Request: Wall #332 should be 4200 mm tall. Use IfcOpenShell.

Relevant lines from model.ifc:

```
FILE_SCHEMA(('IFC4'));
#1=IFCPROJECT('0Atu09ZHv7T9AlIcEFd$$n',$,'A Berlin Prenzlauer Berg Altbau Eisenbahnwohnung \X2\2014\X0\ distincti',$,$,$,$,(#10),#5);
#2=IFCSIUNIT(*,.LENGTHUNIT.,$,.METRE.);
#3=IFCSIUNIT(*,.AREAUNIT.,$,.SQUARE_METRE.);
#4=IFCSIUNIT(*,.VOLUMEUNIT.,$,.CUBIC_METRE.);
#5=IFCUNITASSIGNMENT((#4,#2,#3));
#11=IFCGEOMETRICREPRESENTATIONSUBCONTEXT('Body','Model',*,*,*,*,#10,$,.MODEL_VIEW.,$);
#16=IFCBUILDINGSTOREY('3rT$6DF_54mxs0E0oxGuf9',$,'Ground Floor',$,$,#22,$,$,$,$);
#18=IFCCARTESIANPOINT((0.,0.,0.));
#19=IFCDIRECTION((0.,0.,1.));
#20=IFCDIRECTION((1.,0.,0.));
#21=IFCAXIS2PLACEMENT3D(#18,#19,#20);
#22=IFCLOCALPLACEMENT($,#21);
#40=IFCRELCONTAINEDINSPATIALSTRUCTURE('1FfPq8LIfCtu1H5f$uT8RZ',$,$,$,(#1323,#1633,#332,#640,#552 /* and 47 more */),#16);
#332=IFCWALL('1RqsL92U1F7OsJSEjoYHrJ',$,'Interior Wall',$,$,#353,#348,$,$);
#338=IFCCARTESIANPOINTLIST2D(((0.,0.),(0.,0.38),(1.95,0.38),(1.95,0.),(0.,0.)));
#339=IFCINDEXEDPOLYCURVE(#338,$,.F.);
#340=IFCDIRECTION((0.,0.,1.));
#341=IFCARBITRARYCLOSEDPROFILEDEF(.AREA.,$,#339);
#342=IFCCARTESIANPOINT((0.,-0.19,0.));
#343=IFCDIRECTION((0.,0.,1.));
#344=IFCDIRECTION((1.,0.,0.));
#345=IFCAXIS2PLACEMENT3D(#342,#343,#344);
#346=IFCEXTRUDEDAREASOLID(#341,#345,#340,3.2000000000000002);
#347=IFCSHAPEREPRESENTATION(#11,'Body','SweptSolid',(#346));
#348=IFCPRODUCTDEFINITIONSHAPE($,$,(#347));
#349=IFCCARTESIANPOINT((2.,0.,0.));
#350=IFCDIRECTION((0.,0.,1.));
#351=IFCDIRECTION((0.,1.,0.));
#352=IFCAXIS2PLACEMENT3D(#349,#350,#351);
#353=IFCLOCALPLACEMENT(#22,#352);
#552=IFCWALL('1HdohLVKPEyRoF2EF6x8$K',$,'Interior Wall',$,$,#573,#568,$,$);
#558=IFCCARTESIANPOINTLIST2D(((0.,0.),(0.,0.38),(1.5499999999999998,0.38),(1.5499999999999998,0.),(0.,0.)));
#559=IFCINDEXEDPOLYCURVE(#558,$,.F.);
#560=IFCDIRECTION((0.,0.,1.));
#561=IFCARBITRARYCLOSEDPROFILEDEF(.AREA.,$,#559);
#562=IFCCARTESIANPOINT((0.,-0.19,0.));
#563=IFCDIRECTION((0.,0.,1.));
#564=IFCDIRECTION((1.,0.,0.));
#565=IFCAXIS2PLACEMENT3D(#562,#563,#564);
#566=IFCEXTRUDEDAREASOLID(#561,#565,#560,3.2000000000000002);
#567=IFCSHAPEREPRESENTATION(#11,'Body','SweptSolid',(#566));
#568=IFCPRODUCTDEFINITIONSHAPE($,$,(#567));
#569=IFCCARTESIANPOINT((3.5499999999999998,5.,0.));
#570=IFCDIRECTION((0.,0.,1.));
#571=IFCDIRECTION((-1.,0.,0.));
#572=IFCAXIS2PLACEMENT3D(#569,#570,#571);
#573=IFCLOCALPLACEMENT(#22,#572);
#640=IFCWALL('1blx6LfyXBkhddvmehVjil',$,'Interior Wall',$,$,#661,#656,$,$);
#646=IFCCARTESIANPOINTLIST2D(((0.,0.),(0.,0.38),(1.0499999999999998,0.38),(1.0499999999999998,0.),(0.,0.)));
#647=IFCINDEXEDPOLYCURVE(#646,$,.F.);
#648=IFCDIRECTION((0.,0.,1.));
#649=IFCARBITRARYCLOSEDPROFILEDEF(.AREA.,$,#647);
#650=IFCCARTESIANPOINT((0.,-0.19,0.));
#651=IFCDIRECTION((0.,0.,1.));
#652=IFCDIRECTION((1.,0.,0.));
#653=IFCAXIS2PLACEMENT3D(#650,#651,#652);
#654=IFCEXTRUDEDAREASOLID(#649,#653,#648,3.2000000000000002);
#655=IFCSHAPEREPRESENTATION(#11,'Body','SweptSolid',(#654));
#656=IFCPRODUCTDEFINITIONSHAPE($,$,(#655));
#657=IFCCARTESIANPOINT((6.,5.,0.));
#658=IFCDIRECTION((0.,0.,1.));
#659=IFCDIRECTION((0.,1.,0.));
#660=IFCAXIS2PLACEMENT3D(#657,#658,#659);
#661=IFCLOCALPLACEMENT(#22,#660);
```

```python
import ifcopenshell
import ifcopenshell.geom
import ifcopenshell.util.representation
import ifcopenshell.util.shape
import ifcopenshell.util.unit

model = ifcopenshell.open("model.ifc")
unit_scale = ifcopenshell.util.unit.calculate_unit_scale(model)
settings = ifcopenshell.geom.settings()


def volume(element):
    """Net volume in cubic metres, openings subtracted."""
    shape = ifcopenshell.geom.create_shape(settings, element)
    return ifcopenshell.util.shape.get_volume(shape.geometry)


wall = model.by_guid("1RqsL92U1F7OsJSEjoYHrJ")
before = volume(wall)

body = ifcopenshell.util.representation.get_representation(wall, "Model", "Body")
solid = body.Items[0]
old_height = solid.Depth
solid.Depth = 4.2 / unit_scale
after = volume(wall)

print(f"height {old_height:g} -> {solid.Depth:g}, volume {before:.3f} -> {after:.3f} m3")

model.write("model_v2.ifc")
```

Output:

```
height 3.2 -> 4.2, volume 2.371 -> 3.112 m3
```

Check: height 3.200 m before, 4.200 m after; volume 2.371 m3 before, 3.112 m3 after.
